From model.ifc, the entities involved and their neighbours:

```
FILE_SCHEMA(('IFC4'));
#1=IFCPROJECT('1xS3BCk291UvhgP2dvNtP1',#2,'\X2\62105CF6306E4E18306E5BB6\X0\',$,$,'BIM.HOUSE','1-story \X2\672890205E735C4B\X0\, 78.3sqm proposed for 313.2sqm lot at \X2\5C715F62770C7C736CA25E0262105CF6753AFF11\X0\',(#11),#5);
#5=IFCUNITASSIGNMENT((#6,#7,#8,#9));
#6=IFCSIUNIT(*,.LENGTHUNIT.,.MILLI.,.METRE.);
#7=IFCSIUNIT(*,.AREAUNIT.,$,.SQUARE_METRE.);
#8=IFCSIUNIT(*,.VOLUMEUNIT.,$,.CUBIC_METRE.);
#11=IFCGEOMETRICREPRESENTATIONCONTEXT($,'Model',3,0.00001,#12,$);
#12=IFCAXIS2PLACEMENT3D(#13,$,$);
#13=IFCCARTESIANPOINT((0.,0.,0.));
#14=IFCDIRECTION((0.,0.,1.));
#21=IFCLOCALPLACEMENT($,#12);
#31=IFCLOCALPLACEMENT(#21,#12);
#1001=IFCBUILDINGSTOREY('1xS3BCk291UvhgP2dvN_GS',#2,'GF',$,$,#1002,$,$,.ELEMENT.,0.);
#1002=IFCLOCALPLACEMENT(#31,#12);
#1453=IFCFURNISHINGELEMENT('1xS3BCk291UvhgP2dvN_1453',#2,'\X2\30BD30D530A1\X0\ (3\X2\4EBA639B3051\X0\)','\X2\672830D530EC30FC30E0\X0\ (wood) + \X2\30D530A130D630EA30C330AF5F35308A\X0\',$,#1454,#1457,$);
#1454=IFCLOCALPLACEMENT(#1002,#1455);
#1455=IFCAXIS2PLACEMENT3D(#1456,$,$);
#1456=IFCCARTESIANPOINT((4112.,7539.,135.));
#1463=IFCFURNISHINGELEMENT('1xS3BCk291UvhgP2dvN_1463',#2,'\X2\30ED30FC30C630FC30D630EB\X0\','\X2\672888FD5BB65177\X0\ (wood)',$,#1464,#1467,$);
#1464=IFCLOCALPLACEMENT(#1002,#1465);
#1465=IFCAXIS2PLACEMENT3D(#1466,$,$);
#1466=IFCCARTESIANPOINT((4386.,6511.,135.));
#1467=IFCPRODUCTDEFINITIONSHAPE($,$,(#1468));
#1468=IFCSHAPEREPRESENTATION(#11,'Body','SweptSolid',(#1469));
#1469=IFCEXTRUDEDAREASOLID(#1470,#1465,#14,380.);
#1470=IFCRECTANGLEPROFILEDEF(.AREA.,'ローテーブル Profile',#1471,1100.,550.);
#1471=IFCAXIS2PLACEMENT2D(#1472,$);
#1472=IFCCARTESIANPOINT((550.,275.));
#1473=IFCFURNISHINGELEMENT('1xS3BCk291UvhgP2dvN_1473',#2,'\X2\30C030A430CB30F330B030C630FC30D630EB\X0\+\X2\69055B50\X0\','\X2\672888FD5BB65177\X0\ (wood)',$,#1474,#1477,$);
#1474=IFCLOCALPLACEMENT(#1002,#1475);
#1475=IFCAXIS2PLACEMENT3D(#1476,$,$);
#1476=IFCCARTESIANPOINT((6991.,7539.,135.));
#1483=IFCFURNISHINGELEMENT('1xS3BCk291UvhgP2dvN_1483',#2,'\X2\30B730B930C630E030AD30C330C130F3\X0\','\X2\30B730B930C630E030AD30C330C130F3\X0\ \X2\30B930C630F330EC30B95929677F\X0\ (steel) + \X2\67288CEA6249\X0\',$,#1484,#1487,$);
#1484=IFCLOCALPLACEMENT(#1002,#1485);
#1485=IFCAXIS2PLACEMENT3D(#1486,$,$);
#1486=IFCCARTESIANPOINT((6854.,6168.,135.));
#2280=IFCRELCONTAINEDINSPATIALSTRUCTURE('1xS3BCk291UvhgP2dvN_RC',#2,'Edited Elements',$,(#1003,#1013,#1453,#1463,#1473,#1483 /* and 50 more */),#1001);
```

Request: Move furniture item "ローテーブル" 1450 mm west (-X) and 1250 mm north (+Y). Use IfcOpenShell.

```python
import ifcopenshell
import ifcopenshell.api.geometry
import ifcopenshell.util.placement

model = ifcopenshell.open("model.ifc")

item = model.by_id(1463)
matrix = ifcopenshell.util.placement.get_local_placement(item.ObjectPlacement)
matrix[0, 3] -= 1450.0
matrix[1, 3] += 1250.0
ifcopenshell.api.geometry.edit_object_placement(model, product=item, matrix=matrix, is_si=False)

print(ifcopenshell.util.placement.get_local_placement(item.ObjectPlacement).round(3) + 0.0)

model.write("model_rev.ifc")
```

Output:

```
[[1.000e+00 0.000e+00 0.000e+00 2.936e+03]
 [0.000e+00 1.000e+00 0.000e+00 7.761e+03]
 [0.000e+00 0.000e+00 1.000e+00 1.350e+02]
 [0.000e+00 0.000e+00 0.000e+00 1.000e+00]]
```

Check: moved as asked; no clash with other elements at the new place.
